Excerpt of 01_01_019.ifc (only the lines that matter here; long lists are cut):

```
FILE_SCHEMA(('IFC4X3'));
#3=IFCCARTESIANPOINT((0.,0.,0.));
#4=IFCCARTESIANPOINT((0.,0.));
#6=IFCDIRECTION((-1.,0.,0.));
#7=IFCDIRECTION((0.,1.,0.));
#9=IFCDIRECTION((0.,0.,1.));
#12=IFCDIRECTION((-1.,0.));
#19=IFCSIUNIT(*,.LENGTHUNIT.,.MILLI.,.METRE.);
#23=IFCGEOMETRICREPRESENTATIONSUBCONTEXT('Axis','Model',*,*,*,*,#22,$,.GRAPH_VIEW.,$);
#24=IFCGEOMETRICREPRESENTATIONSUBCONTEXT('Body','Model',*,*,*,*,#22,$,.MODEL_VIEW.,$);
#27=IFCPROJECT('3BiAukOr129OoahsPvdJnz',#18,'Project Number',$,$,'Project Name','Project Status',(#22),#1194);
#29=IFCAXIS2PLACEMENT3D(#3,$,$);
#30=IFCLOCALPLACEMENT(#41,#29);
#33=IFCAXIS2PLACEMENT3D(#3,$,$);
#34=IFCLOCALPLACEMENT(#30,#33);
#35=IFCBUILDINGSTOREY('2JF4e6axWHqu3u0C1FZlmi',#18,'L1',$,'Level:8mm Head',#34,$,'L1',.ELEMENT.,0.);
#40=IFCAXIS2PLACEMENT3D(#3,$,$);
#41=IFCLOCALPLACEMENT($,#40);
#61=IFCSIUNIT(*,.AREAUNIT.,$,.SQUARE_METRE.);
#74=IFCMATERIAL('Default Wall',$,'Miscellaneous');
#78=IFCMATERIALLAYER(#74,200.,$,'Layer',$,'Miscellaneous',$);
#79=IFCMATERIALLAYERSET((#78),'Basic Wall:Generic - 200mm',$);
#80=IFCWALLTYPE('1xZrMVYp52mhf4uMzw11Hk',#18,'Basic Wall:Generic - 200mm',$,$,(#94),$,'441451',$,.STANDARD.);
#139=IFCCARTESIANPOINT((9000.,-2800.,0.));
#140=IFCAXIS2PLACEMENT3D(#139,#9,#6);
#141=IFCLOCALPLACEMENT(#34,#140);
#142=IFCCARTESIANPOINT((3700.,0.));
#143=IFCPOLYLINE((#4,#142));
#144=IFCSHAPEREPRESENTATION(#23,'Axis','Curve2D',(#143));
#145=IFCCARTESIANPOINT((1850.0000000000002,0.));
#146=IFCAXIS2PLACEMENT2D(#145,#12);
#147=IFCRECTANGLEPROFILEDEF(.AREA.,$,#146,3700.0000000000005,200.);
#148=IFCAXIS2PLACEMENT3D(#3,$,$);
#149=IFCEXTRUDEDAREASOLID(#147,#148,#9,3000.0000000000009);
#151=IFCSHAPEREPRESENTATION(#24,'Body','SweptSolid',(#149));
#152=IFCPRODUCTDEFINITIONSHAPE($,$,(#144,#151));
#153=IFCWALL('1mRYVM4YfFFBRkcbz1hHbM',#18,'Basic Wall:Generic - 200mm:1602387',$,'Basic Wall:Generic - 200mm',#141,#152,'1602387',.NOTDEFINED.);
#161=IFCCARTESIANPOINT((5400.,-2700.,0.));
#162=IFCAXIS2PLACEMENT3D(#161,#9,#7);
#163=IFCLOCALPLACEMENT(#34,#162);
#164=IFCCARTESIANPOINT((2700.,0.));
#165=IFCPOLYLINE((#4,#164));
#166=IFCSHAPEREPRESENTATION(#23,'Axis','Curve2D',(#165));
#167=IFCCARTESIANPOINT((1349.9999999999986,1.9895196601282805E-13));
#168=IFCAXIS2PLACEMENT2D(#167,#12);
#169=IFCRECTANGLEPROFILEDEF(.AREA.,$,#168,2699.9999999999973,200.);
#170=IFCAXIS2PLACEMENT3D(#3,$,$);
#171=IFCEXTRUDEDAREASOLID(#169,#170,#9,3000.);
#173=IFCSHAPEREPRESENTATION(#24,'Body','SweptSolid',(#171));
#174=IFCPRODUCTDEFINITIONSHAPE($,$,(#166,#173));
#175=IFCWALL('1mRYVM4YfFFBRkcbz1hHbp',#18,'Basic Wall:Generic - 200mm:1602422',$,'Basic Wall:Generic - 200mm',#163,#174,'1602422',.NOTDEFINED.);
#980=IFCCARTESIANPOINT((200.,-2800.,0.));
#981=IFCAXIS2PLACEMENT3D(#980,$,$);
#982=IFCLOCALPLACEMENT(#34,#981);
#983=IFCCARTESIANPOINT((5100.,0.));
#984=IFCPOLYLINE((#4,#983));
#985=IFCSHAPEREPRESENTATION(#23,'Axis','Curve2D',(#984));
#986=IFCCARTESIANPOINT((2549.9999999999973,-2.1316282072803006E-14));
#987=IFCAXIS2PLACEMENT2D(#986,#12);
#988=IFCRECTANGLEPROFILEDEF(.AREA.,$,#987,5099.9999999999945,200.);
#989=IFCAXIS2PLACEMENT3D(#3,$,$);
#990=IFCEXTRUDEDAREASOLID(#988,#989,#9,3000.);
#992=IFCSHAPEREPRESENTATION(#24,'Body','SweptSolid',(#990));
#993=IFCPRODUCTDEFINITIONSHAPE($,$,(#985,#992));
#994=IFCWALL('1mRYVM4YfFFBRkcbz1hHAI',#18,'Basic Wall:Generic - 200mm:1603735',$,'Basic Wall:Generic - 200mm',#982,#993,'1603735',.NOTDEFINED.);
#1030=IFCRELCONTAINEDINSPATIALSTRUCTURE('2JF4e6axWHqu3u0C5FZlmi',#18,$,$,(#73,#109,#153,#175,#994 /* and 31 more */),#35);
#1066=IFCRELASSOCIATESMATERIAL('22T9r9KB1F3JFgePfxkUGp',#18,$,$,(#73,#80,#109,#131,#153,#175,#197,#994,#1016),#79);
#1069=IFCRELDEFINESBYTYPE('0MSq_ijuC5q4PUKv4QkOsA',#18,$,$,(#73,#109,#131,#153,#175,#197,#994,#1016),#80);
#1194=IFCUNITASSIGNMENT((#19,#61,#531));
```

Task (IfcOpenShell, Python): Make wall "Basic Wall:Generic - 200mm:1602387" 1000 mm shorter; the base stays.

```python
import ifcopenshell
import ifcopenshell.geom
import ifcopenshell.util.representation
import ifcopenshell.util.shape
import ifcopenshell.util.unit

model = ifcopenshell.open("01_01_019.ifc")
unit_scale = ifcopenshell.util.unit.calculate_unit_scale(model)
settings = ifcopenshell.geom.settings()


def volume(element):
    """Net volume in cubic metres, openings subtracted."""
    shape = ifcopenshell.geom.create_shape(settings, element)
    return ifcopenshell.util.shape.get_volume(shape.geometry)


wall = model.by_id(153)
before = volume(wall)

body = ifcopenshell.util.representation.get_representation(wall, "Model", "Body")
solid = body.Items[0]
old_height = solid.Depth
solid.Depth -= 1 / unit_scale
after = volume(wall)

print(f"height {old_height:g} -> {solid.Depth:g}, volume {before:.3f} -> {after:.3f} m3")

model.write("01_01_019_rev.ifc")
```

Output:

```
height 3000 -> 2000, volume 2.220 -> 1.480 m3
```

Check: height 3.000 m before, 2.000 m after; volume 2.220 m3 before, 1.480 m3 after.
